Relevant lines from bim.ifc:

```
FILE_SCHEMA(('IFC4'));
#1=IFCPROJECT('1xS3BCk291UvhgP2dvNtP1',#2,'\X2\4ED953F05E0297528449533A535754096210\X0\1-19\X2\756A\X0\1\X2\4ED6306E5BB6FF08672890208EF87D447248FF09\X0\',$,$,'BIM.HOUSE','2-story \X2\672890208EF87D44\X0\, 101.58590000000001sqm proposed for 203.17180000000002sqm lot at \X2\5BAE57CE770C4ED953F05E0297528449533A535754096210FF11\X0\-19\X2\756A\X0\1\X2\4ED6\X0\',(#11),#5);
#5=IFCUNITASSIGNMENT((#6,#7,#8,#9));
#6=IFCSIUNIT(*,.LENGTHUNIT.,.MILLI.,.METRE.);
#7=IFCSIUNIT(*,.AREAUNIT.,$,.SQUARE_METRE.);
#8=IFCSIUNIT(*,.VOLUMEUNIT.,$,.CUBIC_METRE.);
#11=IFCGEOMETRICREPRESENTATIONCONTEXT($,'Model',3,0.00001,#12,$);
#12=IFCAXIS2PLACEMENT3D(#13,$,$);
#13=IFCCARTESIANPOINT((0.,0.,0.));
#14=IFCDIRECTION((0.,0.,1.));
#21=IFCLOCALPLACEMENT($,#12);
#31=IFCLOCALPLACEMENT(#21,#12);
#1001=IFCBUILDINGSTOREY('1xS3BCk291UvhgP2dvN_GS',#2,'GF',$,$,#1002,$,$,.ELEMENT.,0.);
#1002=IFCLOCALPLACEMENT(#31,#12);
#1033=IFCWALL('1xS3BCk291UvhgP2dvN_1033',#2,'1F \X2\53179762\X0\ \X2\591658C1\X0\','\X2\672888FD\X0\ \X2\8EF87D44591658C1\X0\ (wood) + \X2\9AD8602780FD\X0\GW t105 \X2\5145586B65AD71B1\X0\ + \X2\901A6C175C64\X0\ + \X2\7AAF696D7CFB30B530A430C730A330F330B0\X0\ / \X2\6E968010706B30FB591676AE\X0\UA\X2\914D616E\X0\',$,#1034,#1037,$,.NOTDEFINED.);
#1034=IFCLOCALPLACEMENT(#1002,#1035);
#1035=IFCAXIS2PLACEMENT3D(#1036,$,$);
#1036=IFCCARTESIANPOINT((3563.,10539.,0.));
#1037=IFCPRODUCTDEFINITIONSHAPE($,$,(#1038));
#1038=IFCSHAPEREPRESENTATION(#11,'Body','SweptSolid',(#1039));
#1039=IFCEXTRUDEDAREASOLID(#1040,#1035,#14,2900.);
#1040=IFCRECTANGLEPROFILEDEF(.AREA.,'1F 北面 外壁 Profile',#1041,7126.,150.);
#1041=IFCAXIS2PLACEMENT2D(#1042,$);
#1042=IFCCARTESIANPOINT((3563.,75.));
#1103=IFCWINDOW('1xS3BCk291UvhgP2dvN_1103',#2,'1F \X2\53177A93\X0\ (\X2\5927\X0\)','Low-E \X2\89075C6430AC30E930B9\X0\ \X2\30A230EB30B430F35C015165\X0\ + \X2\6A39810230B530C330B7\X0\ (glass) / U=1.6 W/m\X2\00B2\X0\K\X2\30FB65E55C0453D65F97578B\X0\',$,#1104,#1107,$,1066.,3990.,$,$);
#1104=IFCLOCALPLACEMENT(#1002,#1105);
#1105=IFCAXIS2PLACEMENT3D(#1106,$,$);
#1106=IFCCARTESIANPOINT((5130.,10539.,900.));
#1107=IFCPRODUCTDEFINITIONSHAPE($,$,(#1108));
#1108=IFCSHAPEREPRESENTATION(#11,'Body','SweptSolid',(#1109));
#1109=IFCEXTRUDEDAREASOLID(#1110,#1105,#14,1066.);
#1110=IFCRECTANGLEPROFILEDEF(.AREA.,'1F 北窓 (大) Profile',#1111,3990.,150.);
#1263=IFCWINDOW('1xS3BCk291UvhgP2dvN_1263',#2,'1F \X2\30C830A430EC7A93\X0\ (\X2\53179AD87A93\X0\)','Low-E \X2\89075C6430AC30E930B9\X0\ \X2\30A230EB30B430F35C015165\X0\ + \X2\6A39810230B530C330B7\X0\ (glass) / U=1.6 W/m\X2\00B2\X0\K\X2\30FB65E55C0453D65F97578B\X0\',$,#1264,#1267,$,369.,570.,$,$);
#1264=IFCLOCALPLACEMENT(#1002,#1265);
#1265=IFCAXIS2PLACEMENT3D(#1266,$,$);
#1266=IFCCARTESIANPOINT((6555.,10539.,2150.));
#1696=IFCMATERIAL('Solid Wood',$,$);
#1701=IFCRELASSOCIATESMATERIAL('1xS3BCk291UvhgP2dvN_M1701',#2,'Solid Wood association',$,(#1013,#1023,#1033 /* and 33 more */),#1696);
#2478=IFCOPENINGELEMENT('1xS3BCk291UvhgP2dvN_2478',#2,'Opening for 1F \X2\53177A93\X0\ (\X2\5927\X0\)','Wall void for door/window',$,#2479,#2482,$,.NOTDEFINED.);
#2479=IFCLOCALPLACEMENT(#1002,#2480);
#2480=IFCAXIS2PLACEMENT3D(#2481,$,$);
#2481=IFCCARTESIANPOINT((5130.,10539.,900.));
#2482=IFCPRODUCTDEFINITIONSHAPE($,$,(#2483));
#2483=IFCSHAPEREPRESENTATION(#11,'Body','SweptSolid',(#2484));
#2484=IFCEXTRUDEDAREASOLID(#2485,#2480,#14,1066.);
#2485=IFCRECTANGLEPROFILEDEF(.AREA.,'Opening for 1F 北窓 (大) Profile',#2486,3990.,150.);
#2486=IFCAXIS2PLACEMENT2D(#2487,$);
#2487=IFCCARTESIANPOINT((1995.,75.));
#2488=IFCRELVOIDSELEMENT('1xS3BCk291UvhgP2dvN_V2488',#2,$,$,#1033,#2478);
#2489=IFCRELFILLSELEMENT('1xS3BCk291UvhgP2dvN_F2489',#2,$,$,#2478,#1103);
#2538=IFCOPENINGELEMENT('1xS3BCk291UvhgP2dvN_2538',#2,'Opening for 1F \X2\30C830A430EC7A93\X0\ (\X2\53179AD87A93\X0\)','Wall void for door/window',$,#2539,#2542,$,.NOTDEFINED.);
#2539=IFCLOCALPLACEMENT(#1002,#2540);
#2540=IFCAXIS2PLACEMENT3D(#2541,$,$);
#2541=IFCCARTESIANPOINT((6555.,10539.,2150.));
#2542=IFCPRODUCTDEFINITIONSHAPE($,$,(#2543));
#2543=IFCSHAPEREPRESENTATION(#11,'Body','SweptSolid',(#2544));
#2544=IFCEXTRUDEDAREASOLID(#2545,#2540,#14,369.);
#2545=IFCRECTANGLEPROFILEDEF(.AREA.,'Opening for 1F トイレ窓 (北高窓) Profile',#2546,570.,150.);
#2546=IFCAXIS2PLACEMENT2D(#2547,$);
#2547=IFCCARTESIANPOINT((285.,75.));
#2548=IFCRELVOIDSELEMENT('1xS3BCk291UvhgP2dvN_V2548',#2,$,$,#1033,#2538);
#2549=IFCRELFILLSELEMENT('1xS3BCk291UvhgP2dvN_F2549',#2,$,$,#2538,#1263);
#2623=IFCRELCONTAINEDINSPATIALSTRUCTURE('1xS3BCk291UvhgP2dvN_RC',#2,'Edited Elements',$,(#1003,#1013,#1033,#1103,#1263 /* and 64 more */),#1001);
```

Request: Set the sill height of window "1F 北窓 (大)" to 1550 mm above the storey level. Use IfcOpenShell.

```python
import numpy as np
import ifcopenshell
import ifcopenshell.api.geometry
import ifcopenshell.geom
import ifcopenshell.util.element
import ifcopenshell.util.placement
import ifcopenshell.util.shape
import ifcopenshell.util.unit

model = ifcopenshell.open("bim.ifc")
unit_scale = ifcopenshell.util.unit.calculate_unit_scale(model)

window = model.by_guid("1xS3BCk291UvhgP2dvN_1103")
opening = window.FillsVoids[0].RelatingOpeningElement
storey = ifcopenshell.util.element.get_container(window, ifc_class="IfcBuildingStorey")
level = ifcopenshell.util.placement.get_local_placement(storey.ObjectPlacement)[2, 3]

# The opening's origin need not be at the sill, so measure its lowest point.
shape = ifcopenshell.geom.create_shape(ifcopenshell.geom.settings(), opening)
bottom = ifcopenshell.util.shape.get_shape_bottom_elevation(shape, shape.geometry) / unit_scale
dz = level + 1.55 / unit_scale - bottom

shift = np.array([0.0, 0.0, dz])
# The window is not placed relative to its opening, so move both.
for product in (opening, window):
    matrix = ifcopenshell.util.placement.get_local_placement(product.ObjectPlacement)
    matrix[:3, 3] += shift
    ifcopenshell.api.geometry.edit_object_placement(model, product=product, matrix=matrix, is_si=False)

print(f"moved by {dz * unit_scale:+.3f} m")

model.write("bim_v2.ifc")
```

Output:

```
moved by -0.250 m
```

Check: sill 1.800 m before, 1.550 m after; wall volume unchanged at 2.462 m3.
